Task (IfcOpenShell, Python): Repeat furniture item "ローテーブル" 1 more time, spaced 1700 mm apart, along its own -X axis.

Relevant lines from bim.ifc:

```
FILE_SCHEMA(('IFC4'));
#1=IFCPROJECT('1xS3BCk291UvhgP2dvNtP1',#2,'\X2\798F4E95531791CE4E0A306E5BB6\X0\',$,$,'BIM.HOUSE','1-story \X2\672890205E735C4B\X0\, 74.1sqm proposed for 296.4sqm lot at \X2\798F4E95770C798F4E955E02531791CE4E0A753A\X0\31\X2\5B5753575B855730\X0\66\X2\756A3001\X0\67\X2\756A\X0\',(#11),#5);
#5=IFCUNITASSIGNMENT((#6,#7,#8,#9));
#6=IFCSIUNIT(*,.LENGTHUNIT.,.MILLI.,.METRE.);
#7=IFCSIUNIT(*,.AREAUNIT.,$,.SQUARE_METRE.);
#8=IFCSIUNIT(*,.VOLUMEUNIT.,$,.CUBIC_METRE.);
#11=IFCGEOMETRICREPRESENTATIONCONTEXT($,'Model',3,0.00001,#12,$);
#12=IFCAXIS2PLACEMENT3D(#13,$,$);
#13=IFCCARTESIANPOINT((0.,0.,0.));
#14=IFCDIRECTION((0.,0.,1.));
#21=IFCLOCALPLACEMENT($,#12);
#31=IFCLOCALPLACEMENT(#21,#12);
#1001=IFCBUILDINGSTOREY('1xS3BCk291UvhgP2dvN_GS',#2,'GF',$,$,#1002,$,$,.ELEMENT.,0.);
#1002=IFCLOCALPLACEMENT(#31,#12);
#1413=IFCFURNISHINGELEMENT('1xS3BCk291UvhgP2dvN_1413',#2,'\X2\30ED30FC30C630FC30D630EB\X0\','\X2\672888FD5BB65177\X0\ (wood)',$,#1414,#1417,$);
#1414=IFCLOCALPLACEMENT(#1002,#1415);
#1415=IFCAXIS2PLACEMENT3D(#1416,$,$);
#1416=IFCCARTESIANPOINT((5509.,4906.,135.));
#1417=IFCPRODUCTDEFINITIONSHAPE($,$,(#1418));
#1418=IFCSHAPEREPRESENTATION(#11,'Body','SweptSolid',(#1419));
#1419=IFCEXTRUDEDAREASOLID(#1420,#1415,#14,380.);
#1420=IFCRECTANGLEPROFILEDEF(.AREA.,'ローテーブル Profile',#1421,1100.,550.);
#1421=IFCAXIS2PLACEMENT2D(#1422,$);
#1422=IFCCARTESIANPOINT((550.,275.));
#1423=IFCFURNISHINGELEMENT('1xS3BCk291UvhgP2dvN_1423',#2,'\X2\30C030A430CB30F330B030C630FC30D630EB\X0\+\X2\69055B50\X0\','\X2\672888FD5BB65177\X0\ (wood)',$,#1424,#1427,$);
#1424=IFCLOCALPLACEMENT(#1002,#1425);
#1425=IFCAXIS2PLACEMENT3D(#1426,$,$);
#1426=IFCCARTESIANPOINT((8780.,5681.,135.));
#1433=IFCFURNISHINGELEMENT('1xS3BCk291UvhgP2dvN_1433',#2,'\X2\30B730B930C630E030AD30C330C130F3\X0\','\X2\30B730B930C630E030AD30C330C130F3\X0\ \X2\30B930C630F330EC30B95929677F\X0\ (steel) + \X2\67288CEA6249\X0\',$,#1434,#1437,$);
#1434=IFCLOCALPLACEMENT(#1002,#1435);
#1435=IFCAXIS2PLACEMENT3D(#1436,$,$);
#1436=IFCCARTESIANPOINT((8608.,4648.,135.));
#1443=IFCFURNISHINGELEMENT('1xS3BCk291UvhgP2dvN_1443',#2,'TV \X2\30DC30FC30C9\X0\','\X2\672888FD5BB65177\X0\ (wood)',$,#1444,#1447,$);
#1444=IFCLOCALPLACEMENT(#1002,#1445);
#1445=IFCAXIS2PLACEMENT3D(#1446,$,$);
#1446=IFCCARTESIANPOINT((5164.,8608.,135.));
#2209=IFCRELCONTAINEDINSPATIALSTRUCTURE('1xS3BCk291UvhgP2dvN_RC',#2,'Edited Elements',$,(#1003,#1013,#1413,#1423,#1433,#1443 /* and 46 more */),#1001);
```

```python
import ifcopenshell
import ifcopenshell.api.geometry
import ifcopenshell.api.root
import ifcopenshell.util.element
import ifcopenshell.util.placement
import ifcopenshell.util.unit

model = ifcopenshell.open("bim.ifc")
unit_scale = ifcopenshell.util.unit.calculate_unit_scale(model)


def reuse_history(source, copy):
    """copy_class also copies each property set's owner history, people and application; keep the originals."""
    for rel in copy.IsDefinedBy:
        if rel.is_a("IfcRelDefinesByProperties") and (history := rel.RelatingPropertyDefinition.OwnerHistory):
            rel.RelatingPropertyDefinition.OwnerHistory = source.OwnerHistory
            ifcopenshell.util.element.remove_deep2(model, history)


source = model.by_guid("1xS3BCk291UvhgP2dvN_1413")
base = ifcopenshell.util.placement.get_local_placement(source.ObjectPlacement)
step = -base[:3, 0] * 1.7 / unit_scale

for i in range(1, 2):
    copy = ifcopenshell.api.root.copy_class(model, product=source)
    copy.Representation = ifcopenshell.util.element.copy_deep(
        model, source.Representation, exclude=["IfcGeometricRepresentationContext", "IfcRepresentationMap"]
    )
    reuse_history(source, copy)
    matrix = base.copy()
    matrix[:3, 3] += i * step
    print("added at", matrix[:3, 3].round(3) + 0.0)
    ifcopenshell.api.geometry.edit_object_placement(model, product=copy, matrix=matrix, is_si=False)

model.write("bim_updated.ifc")
```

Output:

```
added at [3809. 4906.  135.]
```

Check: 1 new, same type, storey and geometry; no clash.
